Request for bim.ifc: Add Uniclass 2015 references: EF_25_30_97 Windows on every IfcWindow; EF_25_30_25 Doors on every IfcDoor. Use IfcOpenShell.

First a look at what the model holds.

```python
import ifcopenshell

model = ifcopenshell.open("bim.ifc")
print(model.schema)
print("classifications:", [c.Name for c in model.by_type("IfcClassification")])
for ifc_class in ("IfcDoor", "IfcRoof", "IfcStair", "IfcWall", "IfcWindow"):
    print(ifc_class, len(model.by_type(ifc_class)))
```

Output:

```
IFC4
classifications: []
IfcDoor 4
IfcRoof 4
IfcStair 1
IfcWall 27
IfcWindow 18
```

```python
import ifcopenshell
import ifcopenshell.api.classification

model = ifcopenshell.open("bim.ifc")

system = ifcopenshell.api.classification.add_classification(model, classification="Uniclass 2015")

codes = {
    "IfcWindow": ("EF_25_30_97", "Windows"),
    "IfcDoor": ("EF_25_30_25", "Doors"),
}
for ifc_class, (code, name) in codes.items():
    products = model.by_type(ifc_class)
    ifcopenshell.api.classification.add_reference(
        model, products=products, classification=system, identification=code, name=name
    )
    print(code, len(products))

model.write("bim_updated.ifc")
```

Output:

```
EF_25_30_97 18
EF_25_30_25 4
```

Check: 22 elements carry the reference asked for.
